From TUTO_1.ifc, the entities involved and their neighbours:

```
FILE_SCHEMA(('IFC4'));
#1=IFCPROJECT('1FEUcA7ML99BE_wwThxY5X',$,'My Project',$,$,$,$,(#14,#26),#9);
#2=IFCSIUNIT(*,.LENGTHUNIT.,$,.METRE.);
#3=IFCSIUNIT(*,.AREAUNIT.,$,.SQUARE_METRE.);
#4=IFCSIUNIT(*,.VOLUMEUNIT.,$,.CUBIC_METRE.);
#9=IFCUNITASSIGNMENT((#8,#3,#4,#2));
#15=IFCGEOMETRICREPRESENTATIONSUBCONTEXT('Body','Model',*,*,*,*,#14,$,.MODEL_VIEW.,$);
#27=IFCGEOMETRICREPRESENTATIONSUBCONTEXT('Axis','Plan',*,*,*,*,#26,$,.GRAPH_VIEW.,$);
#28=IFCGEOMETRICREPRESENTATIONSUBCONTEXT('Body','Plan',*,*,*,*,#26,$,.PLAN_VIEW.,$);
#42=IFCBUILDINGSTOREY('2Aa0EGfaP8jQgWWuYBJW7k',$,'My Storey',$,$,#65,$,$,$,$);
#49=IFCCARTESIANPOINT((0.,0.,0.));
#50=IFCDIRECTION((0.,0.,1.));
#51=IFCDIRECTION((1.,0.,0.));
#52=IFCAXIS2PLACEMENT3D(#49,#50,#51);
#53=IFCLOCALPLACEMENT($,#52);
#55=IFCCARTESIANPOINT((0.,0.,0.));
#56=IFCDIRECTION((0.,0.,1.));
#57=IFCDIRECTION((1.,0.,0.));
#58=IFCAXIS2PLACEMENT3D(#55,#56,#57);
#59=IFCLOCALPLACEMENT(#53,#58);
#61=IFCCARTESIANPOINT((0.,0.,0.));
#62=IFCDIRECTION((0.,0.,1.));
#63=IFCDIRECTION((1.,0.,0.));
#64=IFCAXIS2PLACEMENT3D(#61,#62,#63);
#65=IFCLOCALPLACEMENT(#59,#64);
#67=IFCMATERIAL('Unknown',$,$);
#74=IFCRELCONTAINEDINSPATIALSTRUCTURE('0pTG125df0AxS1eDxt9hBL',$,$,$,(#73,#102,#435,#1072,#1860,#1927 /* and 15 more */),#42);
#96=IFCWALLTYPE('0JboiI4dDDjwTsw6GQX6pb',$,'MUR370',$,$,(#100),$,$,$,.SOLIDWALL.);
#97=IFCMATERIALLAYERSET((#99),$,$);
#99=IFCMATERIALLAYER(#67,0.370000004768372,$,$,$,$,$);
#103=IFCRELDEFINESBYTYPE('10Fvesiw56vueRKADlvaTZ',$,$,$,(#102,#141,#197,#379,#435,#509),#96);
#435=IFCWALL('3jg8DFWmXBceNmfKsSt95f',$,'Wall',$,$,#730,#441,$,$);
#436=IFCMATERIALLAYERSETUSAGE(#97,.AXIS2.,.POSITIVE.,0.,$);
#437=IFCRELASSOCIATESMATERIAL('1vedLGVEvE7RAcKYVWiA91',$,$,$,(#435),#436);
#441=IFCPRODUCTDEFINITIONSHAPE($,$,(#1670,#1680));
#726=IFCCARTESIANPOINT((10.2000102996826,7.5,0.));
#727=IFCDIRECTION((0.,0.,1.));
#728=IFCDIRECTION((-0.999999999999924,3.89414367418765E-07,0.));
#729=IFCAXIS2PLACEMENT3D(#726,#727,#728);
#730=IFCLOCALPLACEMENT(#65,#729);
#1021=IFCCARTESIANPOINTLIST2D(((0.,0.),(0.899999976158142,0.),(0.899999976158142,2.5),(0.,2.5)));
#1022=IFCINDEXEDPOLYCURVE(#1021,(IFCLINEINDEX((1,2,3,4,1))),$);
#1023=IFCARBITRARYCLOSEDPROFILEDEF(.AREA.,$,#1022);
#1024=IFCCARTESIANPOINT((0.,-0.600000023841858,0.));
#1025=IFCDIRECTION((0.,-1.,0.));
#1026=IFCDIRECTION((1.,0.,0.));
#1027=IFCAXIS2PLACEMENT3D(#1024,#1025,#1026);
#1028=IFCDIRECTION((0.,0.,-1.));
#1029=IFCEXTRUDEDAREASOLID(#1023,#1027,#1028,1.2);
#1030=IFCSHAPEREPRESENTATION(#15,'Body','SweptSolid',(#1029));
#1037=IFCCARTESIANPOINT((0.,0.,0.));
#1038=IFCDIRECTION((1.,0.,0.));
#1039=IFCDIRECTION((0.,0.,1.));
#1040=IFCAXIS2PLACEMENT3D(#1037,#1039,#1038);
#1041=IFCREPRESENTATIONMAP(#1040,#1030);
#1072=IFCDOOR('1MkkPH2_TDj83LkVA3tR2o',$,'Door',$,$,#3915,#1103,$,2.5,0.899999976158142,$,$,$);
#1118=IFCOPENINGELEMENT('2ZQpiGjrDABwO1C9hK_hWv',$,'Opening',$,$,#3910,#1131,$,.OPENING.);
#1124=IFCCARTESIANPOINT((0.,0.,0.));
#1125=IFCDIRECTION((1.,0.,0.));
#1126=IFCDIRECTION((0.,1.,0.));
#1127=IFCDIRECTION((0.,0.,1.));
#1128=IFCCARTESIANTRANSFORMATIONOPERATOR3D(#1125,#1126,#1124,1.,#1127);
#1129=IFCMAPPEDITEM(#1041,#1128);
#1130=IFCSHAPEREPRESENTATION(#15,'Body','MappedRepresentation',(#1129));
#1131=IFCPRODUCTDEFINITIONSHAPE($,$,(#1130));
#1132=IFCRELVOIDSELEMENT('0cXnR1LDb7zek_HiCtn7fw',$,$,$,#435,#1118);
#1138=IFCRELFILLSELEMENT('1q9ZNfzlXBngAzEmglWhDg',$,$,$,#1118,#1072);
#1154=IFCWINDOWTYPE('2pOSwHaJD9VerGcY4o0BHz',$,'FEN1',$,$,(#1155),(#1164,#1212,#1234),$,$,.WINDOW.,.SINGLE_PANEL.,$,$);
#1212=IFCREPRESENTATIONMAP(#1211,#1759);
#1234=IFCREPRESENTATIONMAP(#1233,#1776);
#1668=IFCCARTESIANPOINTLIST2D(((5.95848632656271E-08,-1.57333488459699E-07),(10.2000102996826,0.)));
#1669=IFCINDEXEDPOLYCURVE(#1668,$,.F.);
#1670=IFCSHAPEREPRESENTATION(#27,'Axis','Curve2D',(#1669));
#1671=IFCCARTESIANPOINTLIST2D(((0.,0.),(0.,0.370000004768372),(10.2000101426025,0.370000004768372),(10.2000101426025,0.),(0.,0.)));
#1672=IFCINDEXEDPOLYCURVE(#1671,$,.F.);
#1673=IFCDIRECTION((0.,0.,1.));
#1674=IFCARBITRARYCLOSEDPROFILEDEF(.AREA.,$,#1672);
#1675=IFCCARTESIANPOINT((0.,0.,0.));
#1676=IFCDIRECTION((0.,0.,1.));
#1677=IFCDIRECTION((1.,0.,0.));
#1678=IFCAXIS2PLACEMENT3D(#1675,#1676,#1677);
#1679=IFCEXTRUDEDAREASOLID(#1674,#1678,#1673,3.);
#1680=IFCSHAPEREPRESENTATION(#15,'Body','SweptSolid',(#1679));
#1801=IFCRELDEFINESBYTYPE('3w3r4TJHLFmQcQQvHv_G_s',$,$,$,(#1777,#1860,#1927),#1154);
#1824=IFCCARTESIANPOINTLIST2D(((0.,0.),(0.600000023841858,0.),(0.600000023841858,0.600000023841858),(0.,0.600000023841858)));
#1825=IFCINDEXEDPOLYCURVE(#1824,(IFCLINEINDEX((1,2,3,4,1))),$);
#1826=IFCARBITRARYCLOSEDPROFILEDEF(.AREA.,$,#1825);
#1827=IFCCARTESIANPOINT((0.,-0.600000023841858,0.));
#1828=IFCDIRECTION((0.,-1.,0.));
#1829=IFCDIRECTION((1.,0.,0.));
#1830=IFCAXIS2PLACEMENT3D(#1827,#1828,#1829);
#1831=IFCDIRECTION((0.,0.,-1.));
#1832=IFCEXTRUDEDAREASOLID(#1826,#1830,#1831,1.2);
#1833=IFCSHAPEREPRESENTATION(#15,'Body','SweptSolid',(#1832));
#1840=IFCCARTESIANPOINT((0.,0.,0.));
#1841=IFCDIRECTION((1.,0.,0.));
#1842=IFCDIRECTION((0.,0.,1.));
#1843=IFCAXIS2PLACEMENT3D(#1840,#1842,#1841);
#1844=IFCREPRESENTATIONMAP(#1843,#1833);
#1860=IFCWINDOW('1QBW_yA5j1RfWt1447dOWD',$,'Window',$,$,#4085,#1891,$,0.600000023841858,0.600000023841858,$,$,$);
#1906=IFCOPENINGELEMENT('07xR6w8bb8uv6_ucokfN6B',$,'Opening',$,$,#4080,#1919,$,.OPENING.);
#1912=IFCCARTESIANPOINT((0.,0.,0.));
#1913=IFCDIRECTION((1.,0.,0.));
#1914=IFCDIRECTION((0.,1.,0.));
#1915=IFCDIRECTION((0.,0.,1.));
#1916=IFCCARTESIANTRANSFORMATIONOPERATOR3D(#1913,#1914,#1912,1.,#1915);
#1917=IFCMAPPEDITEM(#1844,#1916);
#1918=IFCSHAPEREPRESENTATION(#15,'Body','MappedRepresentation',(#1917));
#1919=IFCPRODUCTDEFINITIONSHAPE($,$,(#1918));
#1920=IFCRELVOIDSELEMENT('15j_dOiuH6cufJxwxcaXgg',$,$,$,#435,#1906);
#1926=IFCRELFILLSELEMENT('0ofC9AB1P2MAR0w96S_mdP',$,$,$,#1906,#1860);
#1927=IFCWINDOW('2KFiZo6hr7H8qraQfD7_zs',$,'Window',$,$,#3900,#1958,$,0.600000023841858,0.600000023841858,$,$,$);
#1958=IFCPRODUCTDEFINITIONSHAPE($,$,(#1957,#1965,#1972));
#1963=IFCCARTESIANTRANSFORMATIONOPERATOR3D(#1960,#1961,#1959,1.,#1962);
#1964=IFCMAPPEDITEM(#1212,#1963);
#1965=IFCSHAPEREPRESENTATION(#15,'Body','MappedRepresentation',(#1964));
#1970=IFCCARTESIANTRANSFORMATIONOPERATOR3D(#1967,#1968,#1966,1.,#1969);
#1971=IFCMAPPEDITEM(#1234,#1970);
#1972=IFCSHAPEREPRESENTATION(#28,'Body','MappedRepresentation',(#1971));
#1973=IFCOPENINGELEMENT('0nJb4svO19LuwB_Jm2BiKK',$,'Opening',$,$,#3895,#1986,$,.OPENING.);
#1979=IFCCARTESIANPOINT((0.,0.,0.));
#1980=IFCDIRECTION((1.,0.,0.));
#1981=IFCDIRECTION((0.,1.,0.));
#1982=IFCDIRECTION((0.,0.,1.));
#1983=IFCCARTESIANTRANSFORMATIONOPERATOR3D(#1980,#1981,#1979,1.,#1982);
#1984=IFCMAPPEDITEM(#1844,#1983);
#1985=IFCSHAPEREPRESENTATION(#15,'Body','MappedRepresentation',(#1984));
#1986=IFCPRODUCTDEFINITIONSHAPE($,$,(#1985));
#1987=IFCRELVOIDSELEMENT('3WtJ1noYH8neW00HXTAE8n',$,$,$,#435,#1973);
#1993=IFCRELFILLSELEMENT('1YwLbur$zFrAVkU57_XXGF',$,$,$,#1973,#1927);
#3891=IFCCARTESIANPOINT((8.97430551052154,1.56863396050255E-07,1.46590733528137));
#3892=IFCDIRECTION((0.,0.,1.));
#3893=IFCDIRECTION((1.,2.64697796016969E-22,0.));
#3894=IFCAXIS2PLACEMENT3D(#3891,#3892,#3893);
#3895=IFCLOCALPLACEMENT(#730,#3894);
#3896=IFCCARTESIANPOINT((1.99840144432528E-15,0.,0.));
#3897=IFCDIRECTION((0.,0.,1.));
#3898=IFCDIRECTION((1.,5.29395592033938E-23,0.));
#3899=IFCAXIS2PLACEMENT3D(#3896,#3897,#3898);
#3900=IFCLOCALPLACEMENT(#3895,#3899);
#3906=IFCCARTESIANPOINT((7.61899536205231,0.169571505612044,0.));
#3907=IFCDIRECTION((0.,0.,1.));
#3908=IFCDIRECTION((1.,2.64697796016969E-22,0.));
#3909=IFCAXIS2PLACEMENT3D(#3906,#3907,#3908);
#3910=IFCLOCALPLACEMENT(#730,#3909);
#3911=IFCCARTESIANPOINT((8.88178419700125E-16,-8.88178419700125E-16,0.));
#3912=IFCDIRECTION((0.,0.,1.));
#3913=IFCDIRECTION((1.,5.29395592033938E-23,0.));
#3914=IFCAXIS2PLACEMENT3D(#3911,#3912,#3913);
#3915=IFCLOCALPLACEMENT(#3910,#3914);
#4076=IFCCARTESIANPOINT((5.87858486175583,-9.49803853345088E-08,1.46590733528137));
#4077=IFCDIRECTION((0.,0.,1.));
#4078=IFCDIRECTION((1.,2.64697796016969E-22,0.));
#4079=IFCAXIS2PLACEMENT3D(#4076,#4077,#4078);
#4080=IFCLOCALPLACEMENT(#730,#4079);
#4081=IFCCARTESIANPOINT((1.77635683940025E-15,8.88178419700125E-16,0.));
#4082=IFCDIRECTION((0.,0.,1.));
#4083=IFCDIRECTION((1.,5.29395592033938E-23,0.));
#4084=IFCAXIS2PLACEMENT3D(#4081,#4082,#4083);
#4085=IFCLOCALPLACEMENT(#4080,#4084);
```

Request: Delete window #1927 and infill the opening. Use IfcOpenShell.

```python
import ifcopenshell
import ifcopenshell.api.feature
import ifcopenshell.api.root
import ifcopenshell.geom
import ifcopenshell.util.shape

model = ifcopenshell.open("TUTO_1.ifc")
settings = ifcopenshell.geom.settings()


def volume(element):
    """Net volume in cubic metres, openings subtracted."""
    shape = ifcopenshell.geom.create_shape(settings, element)
    return ifcopenshell.util.shape.get_volume(shape.geometry)


window = model.by_guid("2KFiZo6hr7H8qraQfD7_zs")
opening = window.FillsVoids[0].RelatingOpeningElement
wall = opening.VoidsElements[0].RelatingBuildingElement
before = volume(wall)

ifcopenshell.api.root.remove_product(model, product=window)
ifcopenshell.api.feature.remove_feature(model, feature=opening)

after = volume(wall)

print(f"wall volume {before:.3f} -> {after:.3f} m3")

model.write("TUTO_1-out.ifc")
```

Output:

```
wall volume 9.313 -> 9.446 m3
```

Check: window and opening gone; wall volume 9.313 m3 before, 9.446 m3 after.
